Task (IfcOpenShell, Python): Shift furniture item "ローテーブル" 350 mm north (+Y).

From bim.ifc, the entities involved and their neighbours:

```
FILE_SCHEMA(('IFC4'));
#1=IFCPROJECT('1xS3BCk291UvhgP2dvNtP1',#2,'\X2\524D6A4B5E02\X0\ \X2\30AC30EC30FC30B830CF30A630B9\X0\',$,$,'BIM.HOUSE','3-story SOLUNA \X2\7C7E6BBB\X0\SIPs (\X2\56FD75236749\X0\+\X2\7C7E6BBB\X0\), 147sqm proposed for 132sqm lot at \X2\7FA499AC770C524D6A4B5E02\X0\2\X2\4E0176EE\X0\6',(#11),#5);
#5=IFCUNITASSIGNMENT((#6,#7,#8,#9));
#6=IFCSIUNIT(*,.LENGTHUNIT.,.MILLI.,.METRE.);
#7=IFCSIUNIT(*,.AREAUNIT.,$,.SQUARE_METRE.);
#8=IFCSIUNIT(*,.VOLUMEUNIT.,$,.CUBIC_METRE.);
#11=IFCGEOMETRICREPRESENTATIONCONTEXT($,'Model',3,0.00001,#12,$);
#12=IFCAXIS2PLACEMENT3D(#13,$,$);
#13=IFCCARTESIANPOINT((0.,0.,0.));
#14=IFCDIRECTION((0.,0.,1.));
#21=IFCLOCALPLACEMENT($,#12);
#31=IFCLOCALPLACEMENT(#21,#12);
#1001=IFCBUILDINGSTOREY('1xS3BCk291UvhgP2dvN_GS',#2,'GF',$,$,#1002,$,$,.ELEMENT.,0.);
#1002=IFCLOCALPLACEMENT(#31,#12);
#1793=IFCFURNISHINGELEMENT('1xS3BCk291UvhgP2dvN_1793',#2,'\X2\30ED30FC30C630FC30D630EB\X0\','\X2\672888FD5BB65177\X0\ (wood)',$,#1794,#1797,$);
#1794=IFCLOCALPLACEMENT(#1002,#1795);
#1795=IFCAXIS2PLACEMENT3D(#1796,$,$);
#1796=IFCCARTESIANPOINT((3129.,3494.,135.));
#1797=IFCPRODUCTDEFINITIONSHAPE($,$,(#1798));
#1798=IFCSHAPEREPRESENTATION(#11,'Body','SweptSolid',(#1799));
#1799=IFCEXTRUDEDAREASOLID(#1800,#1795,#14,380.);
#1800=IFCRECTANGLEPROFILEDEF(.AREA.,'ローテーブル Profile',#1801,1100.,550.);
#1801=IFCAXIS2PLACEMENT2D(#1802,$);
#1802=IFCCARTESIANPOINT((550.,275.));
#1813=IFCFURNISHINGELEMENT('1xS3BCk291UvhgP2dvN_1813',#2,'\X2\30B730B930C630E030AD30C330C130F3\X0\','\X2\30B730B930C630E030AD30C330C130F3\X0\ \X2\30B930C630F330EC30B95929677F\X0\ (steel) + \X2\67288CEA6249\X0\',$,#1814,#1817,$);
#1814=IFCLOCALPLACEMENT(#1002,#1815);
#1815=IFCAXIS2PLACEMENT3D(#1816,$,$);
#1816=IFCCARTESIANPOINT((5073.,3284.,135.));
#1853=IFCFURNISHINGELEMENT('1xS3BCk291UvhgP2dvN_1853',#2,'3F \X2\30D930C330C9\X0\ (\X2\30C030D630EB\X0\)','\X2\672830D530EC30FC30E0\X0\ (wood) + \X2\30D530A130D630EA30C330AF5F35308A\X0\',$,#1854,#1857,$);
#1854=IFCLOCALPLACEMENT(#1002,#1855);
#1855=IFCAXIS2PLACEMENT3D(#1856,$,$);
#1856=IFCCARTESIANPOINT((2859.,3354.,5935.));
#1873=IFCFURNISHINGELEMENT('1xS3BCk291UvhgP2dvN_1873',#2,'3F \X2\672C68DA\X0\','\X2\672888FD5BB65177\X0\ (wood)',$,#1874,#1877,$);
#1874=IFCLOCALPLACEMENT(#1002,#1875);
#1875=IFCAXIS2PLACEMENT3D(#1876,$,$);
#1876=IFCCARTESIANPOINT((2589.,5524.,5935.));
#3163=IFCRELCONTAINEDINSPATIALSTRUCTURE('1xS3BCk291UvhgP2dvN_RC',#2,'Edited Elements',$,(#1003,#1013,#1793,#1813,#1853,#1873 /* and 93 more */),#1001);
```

```python
import ifcopenshell
import ifcopenshell.api.geometry
import ifcopenshell.util.placement
import ifcopenshell.util.unit

model = ifcopenshell.open("bim.ifc")
unit_scale = ifcopenshell.util.unit.calculate_unit_scale(model)

item = model.by_guid("1xS3BCk291UvhgP2dvN_1793")
matrix = ifcopenshell.util.placement.get_local_placement(item.ObjectPlacement)
matrix[1, 3] += 0.35 / unit_scale
ifcopenshell.api.geometry.edit_object_placement(model, product=item, matrix=matrix, is_si=False)

print(ifcopenshell.util.placement.get_local_placement(item.ObjectPlacement).round(3) + 0.0)

model.write("bim_rev.ifc")
```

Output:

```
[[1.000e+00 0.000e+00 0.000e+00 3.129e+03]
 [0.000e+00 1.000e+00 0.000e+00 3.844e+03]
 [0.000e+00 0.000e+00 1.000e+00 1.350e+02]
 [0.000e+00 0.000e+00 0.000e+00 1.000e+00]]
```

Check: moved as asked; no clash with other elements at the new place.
